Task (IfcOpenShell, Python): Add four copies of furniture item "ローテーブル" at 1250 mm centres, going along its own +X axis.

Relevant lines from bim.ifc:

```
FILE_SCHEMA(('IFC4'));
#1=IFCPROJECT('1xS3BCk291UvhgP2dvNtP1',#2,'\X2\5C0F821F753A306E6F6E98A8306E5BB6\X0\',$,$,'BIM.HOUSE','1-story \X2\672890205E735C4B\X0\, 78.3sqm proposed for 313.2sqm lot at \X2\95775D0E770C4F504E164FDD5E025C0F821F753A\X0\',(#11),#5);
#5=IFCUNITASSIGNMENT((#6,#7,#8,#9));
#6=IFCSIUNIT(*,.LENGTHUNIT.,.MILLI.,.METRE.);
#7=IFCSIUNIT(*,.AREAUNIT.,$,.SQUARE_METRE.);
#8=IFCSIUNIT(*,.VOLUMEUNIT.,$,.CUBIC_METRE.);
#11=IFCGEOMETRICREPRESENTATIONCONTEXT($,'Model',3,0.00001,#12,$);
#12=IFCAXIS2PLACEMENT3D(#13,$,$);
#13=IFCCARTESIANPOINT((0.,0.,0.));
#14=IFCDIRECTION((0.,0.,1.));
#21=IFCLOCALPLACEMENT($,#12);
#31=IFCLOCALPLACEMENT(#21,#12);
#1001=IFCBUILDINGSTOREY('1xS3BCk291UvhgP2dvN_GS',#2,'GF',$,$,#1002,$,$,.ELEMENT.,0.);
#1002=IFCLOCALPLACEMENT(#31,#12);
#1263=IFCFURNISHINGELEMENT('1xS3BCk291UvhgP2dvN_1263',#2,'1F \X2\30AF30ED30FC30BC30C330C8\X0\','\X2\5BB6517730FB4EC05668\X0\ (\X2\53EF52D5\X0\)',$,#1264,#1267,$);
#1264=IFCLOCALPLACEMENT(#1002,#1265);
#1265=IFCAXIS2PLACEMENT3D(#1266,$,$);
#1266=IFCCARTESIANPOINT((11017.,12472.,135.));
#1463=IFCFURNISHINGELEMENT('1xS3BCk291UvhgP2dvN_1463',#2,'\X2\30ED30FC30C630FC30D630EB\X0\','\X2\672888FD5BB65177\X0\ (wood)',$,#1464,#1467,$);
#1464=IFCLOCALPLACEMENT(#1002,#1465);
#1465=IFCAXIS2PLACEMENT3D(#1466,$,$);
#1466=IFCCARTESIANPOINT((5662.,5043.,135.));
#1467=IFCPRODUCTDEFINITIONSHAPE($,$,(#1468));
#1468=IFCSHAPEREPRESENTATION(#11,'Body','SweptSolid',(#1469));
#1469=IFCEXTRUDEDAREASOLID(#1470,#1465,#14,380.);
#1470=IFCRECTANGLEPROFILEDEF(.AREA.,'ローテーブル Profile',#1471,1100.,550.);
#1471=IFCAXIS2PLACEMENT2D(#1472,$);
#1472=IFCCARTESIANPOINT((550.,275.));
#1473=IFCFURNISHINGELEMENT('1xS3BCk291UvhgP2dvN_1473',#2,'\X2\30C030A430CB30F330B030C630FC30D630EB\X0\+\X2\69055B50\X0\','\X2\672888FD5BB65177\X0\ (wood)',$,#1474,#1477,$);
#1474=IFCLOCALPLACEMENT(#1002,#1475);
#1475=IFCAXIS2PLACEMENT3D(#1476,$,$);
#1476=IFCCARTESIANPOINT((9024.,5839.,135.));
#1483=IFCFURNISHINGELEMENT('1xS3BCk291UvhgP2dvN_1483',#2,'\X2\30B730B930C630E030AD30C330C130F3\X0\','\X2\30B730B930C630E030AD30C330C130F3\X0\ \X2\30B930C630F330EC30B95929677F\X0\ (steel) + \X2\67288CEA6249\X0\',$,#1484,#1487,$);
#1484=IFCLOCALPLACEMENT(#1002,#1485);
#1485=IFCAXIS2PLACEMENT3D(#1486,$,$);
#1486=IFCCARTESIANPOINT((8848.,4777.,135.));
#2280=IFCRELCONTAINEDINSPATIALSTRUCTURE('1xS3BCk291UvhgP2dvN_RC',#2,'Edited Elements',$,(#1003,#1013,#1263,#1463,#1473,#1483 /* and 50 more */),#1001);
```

```python
import ifcopenshell
import ifcopenshell.api.geometry
import ifcopenshell.api.root
import ifcopenshell.util.element
import ifcopenshell.util.placement

model = ifcopenshell.open("bim.ifc")


def reuse_history(source, copy):
    """copy_class also copies each property set's owner history, people and application; keep the originals."""
    for rel in copy.IsDefinedBy:
        if rel.is_a("IfcRelDefinesByProperties") and (history := rel.RelatingPropertyDefinition.OwnerHistory):
            rel.RelatingPropertyDefinition.OwnerHistory = source.OwnerHistory
            ifcopenshell.util.element.remove_deep2(model, history)


source = model.by_id(1463)
base = ifcopenshell.util.placement.get_local_placement(source.ObjectPlacement)
step = base[:3, 0] * 1250.0

for i in range(1, 5):
    copy = ifcopenshell.api.root.copy_class(model, product=source)
    copy.Representation = ifcopenshell.util.element.copy_deep(
        model, source.Representation, exclude=["IfcGeometricRepresentationContext", "IfcRepresentationMap"]
    )
    reuse_history(source, copy)
    matrix = base.copy()
    matrix[:3, 3] += i * step
    print("added at", matrix[:3, 3].round(3) + 0.0)
    ifcopenshell.api.geometry.edit_object_placement(model, product=copy, matrix=matrix, is_si=False)

model.write("bim_v2.ifc")
```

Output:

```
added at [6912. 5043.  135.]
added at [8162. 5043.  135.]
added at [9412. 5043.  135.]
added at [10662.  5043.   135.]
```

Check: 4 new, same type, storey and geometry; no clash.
